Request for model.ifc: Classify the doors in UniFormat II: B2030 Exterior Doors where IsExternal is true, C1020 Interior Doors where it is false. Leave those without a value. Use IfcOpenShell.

First a look at what the model holds.

```python
import ifcopenshell
import ifcopenshell.util.element

model = ifcopenshell.open("model.ifc")
print(model.schema)
print("classifications:", [c.Name for c in model.by_type("IfcClassification")])
values = [ifcopenshell.util.element.get_pset(e, "Pset_DoorCommon", "IsExternal") for e in model.by_type("IfcDoor")]
for value in (True, False, None):
    print("IsExternal", value, values.count(value))
```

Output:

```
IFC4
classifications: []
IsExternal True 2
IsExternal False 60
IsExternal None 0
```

```python
import ifcopenshell
import ifcopenshell.api.classification
import ifcopenshell.util.element

model = ifcopenshell.open("model.ifc")

system = ifcopenshell.api.classification.add_classification(model, classification="UniFormat II")

doors = model.by_type("IfcDoor")
external = {e: ifcopenshell.util.element.get_pset(e, "Pset_DoorCommon", "IsExternal") for e in doors}
for flag, code, name in ((True, "B2030", "Exterior Doors"), (False, "C1020", "Interior Doors")):
    products = [e for e in doors if external[e] is flag]
    ifcopenshell.api.classification.add_reference(
        model, products=products, classification=system, identification=code, name=name
    )
    print(code, len(products))

model.write("model-out.ifc")
```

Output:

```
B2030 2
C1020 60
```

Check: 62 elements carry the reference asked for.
